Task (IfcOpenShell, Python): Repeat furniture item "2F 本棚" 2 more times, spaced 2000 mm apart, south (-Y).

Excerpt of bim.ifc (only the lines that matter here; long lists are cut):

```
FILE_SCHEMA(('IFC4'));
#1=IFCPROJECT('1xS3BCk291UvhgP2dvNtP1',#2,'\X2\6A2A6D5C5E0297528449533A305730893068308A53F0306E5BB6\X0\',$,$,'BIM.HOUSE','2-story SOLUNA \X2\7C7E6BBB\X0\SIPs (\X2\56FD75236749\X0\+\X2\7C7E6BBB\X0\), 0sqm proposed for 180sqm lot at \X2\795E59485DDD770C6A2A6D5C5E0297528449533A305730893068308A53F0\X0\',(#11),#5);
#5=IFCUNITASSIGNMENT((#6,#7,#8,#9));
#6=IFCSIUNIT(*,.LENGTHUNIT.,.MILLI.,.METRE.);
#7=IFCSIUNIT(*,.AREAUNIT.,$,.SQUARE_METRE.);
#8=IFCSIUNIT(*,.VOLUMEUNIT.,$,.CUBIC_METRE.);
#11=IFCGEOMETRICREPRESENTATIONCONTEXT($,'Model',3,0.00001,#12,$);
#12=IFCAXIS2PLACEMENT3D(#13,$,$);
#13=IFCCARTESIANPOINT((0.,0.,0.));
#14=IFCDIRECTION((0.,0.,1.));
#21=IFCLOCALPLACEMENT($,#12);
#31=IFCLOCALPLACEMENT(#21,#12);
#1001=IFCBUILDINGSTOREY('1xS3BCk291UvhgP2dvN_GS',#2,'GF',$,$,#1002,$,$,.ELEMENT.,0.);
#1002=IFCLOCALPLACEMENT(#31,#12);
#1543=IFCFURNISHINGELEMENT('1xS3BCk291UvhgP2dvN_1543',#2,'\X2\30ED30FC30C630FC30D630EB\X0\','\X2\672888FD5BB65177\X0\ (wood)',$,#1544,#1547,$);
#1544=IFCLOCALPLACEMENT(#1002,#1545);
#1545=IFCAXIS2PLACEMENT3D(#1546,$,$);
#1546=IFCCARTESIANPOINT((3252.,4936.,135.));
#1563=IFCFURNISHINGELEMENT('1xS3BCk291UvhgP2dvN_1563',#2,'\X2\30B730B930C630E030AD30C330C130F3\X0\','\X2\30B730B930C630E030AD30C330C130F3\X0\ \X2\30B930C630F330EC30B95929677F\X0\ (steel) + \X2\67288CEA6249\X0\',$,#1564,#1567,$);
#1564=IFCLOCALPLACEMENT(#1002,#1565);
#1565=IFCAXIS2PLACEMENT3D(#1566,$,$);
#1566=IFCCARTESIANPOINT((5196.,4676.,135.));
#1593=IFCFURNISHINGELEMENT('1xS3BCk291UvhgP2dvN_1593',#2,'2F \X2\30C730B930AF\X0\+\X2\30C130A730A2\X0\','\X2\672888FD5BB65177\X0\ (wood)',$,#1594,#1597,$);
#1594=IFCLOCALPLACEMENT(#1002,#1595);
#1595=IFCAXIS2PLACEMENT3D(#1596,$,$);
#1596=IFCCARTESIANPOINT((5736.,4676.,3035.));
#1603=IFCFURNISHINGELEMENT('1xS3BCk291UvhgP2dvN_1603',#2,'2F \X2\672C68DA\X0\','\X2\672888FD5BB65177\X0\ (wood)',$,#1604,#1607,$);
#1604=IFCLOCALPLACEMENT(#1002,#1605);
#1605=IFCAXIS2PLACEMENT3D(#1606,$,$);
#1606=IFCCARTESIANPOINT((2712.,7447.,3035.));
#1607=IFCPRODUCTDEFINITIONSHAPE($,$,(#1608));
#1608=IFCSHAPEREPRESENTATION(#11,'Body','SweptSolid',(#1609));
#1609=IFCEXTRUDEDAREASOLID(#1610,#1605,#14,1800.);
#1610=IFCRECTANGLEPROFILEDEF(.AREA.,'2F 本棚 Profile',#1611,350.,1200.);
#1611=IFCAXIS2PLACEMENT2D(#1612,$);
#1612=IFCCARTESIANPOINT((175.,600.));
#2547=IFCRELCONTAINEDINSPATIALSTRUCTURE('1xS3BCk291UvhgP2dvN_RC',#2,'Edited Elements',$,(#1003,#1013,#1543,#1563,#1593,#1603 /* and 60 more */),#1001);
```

```python
import numpy as np
import ifcopenshell
import ifcopenshell.api.geometry
import ifcopenshell.api.root
import ifcopenshell.util.element
import ifcopenshell.util.placement
import ifcopenshell.util.unit

model = ifcopenshell.open("bim.ifc")
unit_scale = ifcopenshell.util.unit.calculate_unit_scale(model)


def reuse_history(source, copy):
    """copy_class also copies each property set's owner history, people and application; keep the originals."""
    for rel in copy.IsDefinedBy:
        if rel.is_a("IfcRelDefinesByProperties") and (history := rel.RelatingPropertyDefinition.OwnerHistory):
            rel.RelatingPropertyDefinition.OwnerHistory = source.OwnerHistory
            ifcopenshell.util.element.remove_deep2(model, history)


source = model.by_guid("1xS3BCk291UvhgP2dvN_1603")
base = ifcopenshell.util.placement.get_local_placement(source.ObjectPlacement)
step = np.array([0.0, -1.0, 0.0]) * 2 / unit_scale

for i in range(1, 3):
    copy = ifcopenshell.api.root.copy_class(model, product=source)
    copy.Representation = ifcopenshell.util.element.copy_deep(
        model, source.Representation, exclude=["IfcGeometricRepresentationContext", "IfcRepresentationMap"]
    )
    reuse_history(source, copy)
    matrix = base.copy()
    matrix[:3, 3] += i * step
    print("added at", matrix[:3, 3].round(3) + 0.0)
    ifcopenshell.api.geometry.edit_object_placement(model, product=copy, matrix=matrix, is_si=False)

model.write("bim_edited.ifc")
```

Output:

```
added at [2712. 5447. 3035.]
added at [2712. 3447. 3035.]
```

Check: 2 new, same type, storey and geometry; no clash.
